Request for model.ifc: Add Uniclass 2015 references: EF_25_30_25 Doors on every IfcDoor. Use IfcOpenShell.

First a look at what the model holds.

```python
import ifcopenshell

model = ifcopenshell.open("model.ifc")
print(model.schema)
print("classifications:", [c.Name for c in model.by_type("IfcClassification")])
for ifc_class in ("IfcDoor", "IfcRoof", "IfcStair", "IfcWall", "IfcWindow"):
    print(ifc_class, len(model.by_type(ifc_class)))
```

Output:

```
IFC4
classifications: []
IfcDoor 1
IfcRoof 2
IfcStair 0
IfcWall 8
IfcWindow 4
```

```python
import ifcopenshell
import ifcopenshell.api.classification

model = ifcopenshell.open("model.ifc")

system = ifcopenshell.api.classification.add_classification(model, classification="Uniclass 2015")

codes = {
    "IfcDoor": ("EF_25_30_25", "Doors"),
}
for ifc_class, (code, name) in codes.items():
    products = model.by_type(ifc_class)
    ifcopenshell.api.classification.add_reference(
        model, products=products, classification=system, identification=code, name=name
    )
    print(code, len(products))

model.write("model-out.ifc")
```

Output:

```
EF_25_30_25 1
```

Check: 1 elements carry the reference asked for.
